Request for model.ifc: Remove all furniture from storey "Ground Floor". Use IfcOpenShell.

First a look at what the model holds.

```python
import ifcopenshell
import ifcopenshell.util.element

model = ifcopenshell.open("model.ifc")
print(model.schema)
storey = next(s for s in model.by_type("IfcBuildingStorey") if s.Name == "Ground Floor")
furniture = [e for e in ifcopenshell.util.element.get_decomposition(storey) if e.is_a("IfcFurnishingElement")]
seen = {}
for e in furniture:
    element_type = ifcopenshell.util.element.get_type(e)
    name = element_type.Name if element_type not in (None, e) else None
    seen[name] = seen.get(name, 0) + 1
for name, count in sorted(seen.items(), key=str):
    print(count, "x", name)
```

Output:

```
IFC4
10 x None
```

```python
import ifcopenshell
import ifcopenshell.api.root
import ifcopenshell.util.element

model = ifcopenshell.open("model.ifc")

storey = next(s for s in model.by_type("IfcBuildingStorey") if s.Name == "Ground Floor")
furniture = [e for e in ifcopenshell.util.element.get_decomposition(storey) if e.is_a("IfcFurnishingElement")]

for e in furniture:
    ifcopenshell.api.root.remove_product(model, product=e)
print(len(furniture), "removed")

model.write("model_rev.ifc")
```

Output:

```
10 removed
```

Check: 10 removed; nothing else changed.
